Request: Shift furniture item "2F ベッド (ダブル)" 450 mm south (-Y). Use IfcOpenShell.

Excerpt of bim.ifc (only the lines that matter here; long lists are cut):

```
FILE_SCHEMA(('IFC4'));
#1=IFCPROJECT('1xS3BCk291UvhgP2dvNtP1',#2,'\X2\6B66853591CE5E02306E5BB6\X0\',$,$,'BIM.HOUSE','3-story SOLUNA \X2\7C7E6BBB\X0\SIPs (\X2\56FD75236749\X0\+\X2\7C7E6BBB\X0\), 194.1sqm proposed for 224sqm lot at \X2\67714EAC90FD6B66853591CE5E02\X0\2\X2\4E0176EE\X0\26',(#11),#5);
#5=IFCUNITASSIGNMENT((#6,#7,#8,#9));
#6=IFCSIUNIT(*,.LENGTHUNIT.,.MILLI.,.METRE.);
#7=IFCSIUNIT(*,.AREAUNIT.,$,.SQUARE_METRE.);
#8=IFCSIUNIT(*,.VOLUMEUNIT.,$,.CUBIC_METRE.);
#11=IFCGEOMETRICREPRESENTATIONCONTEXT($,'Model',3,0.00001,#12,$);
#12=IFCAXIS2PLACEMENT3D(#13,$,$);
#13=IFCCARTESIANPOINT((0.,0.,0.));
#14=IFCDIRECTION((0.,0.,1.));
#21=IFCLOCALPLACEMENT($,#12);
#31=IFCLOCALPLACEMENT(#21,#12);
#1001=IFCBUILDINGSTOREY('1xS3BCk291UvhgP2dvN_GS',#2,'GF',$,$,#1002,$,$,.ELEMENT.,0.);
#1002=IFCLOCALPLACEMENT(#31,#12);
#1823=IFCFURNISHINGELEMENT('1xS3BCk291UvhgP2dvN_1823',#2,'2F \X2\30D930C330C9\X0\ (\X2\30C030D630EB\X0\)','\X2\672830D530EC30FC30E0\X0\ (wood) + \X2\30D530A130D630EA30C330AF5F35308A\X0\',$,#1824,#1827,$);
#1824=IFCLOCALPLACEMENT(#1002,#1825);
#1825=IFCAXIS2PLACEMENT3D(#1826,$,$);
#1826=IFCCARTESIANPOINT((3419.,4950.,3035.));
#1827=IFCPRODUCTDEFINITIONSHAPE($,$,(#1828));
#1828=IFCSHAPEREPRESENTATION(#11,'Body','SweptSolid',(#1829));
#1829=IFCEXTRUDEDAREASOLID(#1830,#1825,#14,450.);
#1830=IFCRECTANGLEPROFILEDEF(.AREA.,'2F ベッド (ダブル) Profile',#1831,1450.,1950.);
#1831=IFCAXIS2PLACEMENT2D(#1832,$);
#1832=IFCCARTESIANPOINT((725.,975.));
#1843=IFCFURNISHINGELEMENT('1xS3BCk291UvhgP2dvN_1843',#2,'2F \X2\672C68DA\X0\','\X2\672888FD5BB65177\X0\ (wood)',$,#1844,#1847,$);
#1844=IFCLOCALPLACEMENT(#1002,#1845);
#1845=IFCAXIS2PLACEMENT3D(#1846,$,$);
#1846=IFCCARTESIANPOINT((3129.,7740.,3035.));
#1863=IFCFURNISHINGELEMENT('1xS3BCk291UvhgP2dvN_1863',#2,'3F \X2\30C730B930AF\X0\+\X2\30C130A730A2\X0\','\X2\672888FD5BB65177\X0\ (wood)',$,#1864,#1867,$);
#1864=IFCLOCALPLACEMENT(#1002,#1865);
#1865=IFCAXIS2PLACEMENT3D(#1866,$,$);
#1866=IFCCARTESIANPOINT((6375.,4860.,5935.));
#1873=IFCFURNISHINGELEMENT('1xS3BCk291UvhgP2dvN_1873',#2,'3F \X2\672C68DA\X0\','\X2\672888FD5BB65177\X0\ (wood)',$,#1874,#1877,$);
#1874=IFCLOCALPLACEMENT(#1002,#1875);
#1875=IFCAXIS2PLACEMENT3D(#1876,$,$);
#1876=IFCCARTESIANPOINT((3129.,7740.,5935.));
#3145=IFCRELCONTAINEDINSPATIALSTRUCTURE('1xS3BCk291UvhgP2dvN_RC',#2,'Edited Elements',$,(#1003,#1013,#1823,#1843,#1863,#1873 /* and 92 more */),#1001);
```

```python
import ifcopenshell
import ifcopenshell.api.geometry
import ifcopenshell.util.placement

model = ifcopenshell.open("bim.ifc")

item = model.by_guid("1xS3BCk291UvhgP2dvN_1823")
matrix = ifcopenshell.util.placement.get_local_placement(item.ObjectPlacement)
matrix[1, 3] -= 450.0
ifcopenshell.api.geometry.edit_object_placement(model, product=item, matrix=matrix, is_si=False)

print(ifcopenshell.util.placement.get_local_placement(item.ObjectPlacement).round(3) + 0.0)

model.write("bim_edited.ifc")
```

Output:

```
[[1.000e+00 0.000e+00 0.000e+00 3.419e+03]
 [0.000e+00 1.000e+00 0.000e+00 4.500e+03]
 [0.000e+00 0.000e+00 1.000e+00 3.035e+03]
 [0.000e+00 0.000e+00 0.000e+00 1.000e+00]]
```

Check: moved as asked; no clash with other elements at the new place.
